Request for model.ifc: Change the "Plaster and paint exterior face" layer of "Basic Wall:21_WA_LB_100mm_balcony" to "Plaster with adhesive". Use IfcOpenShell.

First a look at what the model holds.

```python
import ifcopenshell
import ifcopenshell.util.element

model = ifcopenshell.open("model.ifc")
print(model.schema)
for layer_set in model.by_type("IfcMaterialLayerSet"):
    if layer_set.LayerSetName == "Basic Wall:21_WA_LB_100mm_balcony":
        for layer in layer_set.MaterialLayers:
            print(layer.id(), layer.Material and layer.Material.Name, layer.LayerThickness, sep=" | ")
        print(len(ifcopenshell.util.element.get_elements_by_material(model, layer_set)), "elements and types use it")
print(sorted(m.Name for m in model.by_type("IfcMaterial") if m.Name)[:60])
```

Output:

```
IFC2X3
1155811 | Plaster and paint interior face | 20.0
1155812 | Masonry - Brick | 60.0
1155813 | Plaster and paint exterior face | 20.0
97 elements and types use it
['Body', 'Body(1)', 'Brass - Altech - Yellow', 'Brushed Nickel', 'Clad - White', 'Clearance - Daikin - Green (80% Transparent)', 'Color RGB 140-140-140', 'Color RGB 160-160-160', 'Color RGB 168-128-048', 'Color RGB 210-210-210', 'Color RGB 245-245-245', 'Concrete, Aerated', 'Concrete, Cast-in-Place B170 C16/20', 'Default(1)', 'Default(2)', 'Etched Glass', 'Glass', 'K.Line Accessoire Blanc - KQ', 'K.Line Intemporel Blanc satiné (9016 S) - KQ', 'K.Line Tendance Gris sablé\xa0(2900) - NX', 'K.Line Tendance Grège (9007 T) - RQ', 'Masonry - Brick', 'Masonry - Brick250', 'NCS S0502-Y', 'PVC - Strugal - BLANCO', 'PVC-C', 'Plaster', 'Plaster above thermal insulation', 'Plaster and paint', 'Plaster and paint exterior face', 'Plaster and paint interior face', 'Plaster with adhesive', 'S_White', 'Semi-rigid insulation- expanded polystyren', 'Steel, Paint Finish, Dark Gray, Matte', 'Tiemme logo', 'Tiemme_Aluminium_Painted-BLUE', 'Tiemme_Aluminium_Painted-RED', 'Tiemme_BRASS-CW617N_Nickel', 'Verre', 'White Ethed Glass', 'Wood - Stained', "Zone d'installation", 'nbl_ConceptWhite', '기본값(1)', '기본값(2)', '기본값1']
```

```python
import ifcopenshell
import ifcopenshell.api.material

model = ifcopenshell.open("model.ifc")

layer_set = next(s for s in model.by_type("IfcMaterialLayerSet") if s.LayerSetName == "Basic Wall:21_WA_LB_100mm_balcony")
layer = next(l for l in layer_set.MaterialLayers if l.Material and l.Material.Name == "Plaster and paint exterior face")
material = next(m for m in model.by_type("IfcMaterial") if m.Name == "Plaster with adhesive")

# Point this one layer at the other material; renaming the old one would change it everywhere.
ifcopenshell.api.material.edit_layer(model, layer=layer, attributes={}, material=material)

print([l.Material.Name if l.Material else None for l in layer_set.MaterialLayers])

model.write("model-out.ifc")
```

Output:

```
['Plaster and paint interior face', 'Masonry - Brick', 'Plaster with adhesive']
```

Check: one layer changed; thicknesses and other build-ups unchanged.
